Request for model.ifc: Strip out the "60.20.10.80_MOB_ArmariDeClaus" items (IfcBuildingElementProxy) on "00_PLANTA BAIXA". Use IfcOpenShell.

First a look at what the model holds.

```python
import ifcopenshell
import ifcopenshell.util.element

model = ifcopenshell.open("model.ifc")
print(model.schema)
storey = next(s for s in model.by_type("IfcBuildingStorey") if s.Name == "00_PLANTA BAIXA")
proxies = [e for e in ifcopenshell.util.element.get_decomposition(storey) if e.is_a("IfcBuildingElementProxy")]
seen = {}
for e in proxies:
    element_type = ifcopenshell.util.element.get_type(e)
    name = element_type.Name if element_type not in (None, e) else None
    seen[name] = seen.get(name, 0) + 1
for name, count in sorted(seen.items(), key=str):
    print(count, "x", name)
```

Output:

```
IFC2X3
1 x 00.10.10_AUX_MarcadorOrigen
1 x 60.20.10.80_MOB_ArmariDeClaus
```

```python
import ifcopenshell
import ifcopenshell.api.root
import ifcopenshell.util.element

model = ifcopenshell.open("model.ifc")

storey = next(s for s in model.by_type("IfcBuildingStorey") if s.Name == "00_PLANTA BAIXA")
proxies = [e for e in ifcopenshell.util.element.get_decomposition(storey) if e.is_a("IfcBuildingElementProxy")]
targets = [e for e in proxies if (t := ifcopenshell.util.element.get_type(e)) not in (None, e) and t.Name == "60.20.10.80_MOB_ArmariDeClaus"]

for e in targets:
    ifcopenshell.api.root.remove_product(model, product=e)
print(len(targets), "removed")

model.write("model_v2.ifc")
```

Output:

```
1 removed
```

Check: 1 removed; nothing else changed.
